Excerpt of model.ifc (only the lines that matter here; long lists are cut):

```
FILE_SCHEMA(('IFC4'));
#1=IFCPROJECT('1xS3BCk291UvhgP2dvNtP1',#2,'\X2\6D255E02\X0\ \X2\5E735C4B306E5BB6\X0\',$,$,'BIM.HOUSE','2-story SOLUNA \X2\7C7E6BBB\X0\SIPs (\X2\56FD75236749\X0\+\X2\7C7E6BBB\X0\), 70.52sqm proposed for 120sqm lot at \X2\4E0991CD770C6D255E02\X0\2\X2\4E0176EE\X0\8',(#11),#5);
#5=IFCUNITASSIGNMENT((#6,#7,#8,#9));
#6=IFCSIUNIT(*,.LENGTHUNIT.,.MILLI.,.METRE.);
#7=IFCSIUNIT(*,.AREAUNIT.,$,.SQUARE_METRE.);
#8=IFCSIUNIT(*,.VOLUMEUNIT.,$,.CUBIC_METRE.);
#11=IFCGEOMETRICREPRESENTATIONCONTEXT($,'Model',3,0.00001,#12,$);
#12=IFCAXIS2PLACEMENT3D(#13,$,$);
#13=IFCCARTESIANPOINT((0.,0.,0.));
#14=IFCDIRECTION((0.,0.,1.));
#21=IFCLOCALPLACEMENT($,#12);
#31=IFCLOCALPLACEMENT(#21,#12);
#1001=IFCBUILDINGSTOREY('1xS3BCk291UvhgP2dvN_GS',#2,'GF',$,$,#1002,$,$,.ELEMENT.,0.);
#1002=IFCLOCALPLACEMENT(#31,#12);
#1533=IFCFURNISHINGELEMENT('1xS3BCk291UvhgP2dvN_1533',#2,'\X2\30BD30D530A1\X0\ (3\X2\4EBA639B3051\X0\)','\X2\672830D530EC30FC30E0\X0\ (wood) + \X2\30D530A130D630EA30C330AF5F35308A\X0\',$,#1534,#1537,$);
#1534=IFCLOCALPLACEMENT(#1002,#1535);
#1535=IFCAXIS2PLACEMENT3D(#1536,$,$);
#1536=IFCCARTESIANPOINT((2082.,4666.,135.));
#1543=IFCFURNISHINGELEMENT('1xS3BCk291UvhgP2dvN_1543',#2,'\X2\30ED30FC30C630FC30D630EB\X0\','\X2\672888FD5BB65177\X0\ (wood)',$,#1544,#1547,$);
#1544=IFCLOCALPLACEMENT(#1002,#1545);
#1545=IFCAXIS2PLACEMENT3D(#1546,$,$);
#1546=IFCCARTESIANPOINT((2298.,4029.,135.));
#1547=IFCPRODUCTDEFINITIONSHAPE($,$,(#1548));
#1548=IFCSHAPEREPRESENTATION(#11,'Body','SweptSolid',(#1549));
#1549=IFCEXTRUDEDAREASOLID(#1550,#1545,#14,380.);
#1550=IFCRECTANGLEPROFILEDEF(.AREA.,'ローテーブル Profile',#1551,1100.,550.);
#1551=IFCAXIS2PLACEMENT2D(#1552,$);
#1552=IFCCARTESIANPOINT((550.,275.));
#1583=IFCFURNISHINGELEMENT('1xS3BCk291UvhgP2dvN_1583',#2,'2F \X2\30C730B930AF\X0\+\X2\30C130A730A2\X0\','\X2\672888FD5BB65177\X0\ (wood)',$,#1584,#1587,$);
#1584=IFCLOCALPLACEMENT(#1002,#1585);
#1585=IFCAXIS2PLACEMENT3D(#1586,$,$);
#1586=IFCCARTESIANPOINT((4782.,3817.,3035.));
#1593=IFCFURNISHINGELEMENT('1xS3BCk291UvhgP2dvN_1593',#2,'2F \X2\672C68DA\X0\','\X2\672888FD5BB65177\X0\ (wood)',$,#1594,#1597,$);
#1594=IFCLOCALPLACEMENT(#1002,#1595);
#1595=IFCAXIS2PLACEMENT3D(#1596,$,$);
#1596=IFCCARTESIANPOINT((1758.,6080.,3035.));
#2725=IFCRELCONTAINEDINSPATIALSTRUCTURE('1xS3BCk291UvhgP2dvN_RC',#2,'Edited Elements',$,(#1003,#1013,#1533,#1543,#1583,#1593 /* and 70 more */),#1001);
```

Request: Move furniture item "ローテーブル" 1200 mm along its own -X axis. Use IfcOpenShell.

```python
import ifcopenshell
import ifcopenshell.api.geometry
import ifcopenshell.util.placement
import ifcopenshell.util.unit

model = ifcopenshell.open("model.ifc")
unit_scale = ifcopenshell.util.unit.calculate_unit_scale(model)

item = model.by_id(1543)
matrix = ifcopenshell.util.placement.get_local_placement(item.ObjectPlacement)
matrix[:3, 3] -= matrix[:3, 0] * 1.2 / unit_scale
ifcopenshell.api.geometry.edit_object_placement(model, product=item, matrix=matrix, is_si=False)

print(ifcopenshell.util.placement.get_local_placement(item.ObjectPlacement).round(3) + 0.0)

model.write("model-out.ifc")
```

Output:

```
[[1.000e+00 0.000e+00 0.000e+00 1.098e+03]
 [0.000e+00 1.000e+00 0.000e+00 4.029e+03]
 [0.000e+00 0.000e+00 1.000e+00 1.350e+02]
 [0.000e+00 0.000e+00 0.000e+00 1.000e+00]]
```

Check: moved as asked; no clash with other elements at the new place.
